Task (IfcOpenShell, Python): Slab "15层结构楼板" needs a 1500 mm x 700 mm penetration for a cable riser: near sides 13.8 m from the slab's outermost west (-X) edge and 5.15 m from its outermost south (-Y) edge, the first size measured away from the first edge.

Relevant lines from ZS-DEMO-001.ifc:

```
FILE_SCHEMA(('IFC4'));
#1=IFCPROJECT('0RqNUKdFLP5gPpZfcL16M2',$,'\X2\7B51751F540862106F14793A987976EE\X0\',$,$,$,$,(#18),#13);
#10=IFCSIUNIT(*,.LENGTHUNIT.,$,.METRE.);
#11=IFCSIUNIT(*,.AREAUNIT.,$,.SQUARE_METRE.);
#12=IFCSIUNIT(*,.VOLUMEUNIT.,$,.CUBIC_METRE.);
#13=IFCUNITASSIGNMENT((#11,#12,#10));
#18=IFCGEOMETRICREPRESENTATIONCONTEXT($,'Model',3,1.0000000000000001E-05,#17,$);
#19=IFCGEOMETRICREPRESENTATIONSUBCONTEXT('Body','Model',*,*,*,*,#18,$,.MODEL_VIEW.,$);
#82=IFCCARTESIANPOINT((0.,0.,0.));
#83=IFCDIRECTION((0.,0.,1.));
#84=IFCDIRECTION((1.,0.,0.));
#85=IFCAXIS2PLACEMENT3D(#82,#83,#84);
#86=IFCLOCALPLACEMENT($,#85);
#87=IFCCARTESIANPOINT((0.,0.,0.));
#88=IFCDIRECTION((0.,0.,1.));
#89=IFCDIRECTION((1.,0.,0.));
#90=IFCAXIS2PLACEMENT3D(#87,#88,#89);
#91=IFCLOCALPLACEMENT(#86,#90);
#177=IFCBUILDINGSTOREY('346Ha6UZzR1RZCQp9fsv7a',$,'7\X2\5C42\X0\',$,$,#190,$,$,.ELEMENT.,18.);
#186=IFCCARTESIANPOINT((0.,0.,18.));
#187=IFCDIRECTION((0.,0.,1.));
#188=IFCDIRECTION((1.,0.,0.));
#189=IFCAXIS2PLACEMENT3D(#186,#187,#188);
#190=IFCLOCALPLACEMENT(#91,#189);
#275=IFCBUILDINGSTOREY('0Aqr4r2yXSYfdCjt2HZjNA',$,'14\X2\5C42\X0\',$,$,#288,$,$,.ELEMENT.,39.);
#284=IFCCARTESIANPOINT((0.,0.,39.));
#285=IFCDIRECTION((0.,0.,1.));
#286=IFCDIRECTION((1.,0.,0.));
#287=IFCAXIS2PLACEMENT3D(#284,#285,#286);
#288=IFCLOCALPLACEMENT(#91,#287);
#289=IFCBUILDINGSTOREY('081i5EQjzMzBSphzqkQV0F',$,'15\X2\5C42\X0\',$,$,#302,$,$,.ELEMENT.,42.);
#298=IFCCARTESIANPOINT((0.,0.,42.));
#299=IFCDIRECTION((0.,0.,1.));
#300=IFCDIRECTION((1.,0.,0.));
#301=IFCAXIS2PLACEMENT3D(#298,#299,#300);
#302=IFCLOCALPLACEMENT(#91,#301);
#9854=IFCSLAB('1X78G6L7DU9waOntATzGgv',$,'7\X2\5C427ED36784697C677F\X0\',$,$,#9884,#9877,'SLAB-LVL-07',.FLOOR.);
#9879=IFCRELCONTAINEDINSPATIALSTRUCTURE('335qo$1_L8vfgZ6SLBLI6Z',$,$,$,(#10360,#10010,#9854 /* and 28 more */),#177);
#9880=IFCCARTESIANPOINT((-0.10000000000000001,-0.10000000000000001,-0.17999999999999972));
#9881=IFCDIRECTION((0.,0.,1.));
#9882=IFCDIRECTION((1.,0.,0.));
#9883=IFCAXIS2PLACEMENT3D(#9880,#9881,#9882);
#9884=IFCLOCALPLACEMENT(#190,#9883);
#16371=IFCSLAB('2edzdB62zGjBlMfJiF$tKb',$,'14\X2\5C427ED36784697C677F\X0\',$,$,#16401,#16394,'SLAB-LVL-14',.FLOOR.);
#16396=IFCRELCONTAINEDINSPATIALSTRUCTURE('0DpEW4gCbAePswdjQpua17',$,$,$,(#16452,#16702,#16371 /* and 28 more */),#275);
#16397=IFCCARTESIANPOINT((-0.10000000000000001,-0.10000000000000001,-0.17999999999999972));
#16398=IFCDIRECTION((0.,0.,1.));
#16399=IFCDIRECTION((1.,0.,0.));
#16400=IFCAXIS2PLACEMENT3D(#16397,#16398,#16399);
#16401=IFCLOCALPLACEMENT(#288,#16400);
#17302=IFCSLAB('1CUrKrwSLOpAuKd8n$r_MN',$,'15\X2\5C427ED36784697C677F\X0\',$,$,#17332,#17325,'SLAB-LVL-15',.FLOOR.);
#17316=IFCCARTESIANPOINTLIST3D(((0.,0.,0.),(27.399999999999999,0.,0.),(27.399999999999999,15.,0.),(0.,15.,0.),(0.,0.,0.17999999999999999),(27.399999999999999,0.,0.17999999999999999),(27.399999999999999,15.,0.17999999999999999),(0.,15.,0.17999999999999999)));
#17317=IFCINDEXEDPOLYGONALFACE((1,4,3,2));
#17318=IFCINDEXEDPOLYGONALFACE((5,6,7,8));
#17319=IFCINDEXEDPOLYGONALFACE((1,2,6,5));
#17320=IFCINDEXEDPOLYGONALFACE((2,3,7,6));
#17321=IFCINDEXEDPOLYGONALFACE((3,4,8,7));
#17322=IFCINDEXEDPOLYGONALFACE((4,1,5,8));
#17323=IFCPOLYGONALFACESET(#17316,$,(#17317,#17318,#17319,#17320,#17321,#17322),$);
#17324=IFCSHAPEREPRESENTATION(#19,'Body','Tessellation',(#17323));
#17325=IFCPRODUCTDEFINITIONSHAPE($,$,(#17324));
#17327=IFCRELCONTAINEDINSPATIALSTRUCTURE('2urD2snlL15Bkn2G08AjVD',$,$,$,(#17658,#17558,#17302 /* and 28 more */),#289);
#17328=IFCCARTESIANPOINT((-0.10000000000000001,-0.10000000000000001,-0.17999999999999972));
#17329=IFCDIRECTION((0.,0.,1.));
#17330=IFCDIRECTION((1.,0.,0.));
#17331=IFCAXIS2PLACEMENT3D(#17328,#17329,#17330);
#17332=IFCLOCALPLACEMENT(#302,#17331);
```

```python
import numpy as np
import ifcopenshell
import ifcopenshell.api.feature
import ifcopenshell.api.geometry
import ifcopenshell.api.root
import ifcopenshell.geom
import ifcopenshell.util.placement
import ifcopenshell.util.representation
import ifcopenshell.util.shape
import ifcopenshell.util.unit

model = ifcopenshell.open("ZS-DEMO-001.ifc")
unit_scale = ifcopenshell.util.unit.calculate_unit_scale(model)
settings = ifcopenshell.geom.settings()


def volume(element):
    """Net volume in cubic metres, openings subtracted."""
    shape = ifcopenshell.geom.create_shape(settings, element)
    return ifcopenshell.util.shape.get_volume(shape.geometry)


slab = model.by_guid("1CUrKrwSLOpAuKd8n$r_MN")
before = volume(slab)

# Extent in the slab's own axes, in metres. The edges named are its -X and -Y sides.
slab_shape = ifcopenshell.geom.create_shape(settings, slab)
vertices = ifcopenshell.util.shape.get_vertices(slab_shape.geometry)
x_min, y_min, bottom = vertices.min(axis=0)
top = vertices[:, 2].max()

opening = ifcopenshell.api.root.create_entity(model, ifc_class="IfcOpeningElement", name="Cable riser opening", predefined_type="OPENING")
context = ifcopenshell.util.representation.get_context(model, "Model", "Body", "MODEL_VIEW")
width, depth = 1.5, 0.7
outline = [(0.0, 0.0), (width, 0.0), (width, depth), (0.0, depth), (0.0, 0.0)]
# Overshoot both faces by 50 mm so the cut is clean.
shape = ifcopenshell.api.geometry.add_slab_representation(
    model, context=context, depth=top - bottom + 0.1, polyline=outline
)
ifcopenshell.api.geometry.assign_representation(model, product=opening, representation=shape)

matrix = ifcopenshell.util.placement.get_local_placement(slab.ObjectPlacement)
matrix[:, 3] = matrix @ np.append(np.array([x_min + 13.8, y_min + 5.15, bottom - 0.05]) / unit_scale, 1.0)
ifcopenshell.api.geometry.edit_object_placement(model, product=opening, matrix=matrix, is_si=False)
ifcopenshell.api.feature.add_feature(model, feature=opening, element=slab)

after = volume(slab)

print(f"slab volume {before:.3f} -> {after:.3f} m3")

model.write("ZS-DEMO-001_updated.ifc")
```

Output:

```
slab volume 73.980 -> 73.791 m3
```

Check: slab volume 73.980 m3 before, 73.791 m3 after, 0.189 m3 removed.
